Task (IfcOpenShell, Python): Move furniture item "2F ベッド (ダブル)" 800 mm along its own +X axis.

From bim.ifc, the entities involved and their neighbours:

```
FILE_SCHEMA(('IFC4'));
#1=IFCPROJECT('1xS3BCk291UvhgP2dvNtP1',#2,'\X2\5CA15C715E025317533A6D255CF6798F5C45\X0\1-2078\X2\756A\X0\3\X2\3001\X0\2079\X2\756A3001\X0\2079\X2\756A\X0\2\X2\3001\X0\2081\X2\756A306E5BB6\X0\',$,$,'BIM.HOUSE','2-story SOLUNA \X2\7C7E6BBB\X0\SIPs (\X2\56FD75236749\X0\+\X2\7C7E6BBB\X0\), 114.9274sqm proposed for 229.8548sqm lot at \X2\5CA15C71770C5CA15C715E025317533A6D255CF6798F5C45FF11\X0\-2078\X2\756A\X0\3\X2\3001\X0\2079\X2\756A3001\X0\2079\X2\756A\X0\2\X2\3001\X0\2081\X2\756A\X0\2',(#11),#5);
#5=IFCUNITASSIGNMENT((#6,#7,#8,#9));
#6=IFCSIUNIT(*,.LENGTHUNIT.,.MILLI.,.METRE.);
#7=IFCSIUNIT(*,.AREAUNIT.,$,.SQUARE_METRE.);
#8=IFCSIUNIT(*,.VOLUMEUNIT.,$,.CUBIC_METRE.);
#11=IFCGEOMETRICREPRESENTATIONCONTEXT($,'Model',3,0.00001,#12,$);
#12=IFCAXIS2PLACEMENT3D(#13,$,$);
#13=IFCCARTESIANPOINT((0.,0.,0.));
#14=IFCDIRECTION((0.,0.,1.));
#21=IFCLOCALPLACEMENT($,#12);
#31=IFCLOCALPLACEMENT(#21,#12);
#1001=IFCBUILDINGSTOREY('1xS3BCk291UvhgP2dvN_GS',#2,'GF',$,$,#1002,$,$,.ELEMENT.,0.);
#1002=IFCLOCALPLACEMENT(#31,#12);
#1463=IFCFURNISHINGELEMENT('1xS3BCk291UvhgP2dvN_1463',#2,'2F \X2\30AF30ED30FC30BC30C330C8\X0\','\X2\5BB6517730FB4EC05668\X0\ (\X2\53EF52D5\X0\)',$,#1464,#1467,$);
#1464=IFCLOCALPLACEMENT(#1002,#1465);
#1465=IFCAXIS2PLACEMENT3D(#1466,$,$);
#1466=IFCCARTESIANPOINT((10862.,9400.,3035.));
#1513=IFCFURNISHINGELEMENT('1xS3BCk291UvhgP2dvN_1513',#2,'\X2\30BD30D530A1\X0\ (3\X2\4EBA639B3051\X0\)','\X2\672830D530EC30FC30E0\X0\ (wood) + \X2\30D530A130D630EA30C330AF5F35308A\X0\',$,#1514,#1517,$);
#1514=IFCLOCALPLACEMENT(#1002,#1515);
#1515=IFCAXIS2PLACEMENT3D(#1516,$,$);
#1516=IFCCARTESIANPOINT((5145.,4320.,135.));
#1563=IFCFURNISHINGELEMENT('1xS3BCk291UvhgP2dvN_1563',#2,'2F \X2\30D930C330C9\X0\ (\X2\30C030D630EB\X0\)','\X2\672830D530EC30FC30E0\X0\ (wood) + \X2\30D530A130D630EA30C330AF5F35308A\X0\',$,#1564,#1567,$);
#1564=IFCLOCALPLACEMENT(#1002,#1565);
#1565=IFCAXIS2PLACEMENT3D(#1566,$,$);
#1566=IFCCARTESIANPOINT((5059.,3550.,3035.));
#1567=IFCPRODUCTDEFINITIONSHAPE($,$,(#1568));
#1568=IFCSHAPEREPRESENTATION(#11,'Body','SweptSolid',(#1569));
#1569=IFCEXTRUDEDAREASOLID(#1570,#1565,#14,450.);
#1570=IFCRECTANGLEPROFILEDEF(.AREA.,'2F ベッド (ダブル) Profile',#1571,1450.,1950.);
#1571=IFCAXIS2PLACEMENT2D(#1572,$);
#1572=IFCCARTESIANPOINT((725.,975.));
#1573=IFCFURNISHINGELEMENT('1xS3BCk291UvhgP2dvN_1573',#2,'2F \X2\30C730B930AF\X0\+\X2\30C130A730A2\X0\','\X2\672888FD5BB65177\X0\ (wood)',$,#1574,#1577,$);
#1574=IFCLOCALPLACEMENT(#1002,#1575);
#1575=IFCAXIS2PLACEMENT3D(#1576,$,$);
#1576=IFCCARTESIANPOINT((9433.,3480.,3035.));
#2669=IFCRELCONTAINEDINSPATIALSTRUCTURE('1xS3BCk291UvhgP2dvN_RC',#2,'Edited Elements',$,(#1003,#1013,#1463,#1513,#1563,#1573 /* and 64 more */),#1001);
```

```python
import ifcopenshell
import ifcopenshell.api.geometry
import ifcopenshell.util.placement
import ifcopenshell.util.unit

model = ifcopenshell.open("bim.ifc")
unit_scale = ifcopenshell.util.unit.calculate_unit_scale(model)

item = model.by_guid("1xS3BCk291UvhgP2dvN_1563")
matrix = ifcopenshell.util.placement.get_local_placement(item.ObjectPlacement)
matrix[:3, 3] += matrix[:3, 0] * 0.8 / unit_scale
ifcopenshell.api.geometry.edit_object_placement(model, product=item, matrix=matrix, is_si=False)

print(ifcopenshell.util.placement.get_local_placement(item.ObjectPlacement).round(3) + 0.0)

model.write("bim_rev.ifc")
```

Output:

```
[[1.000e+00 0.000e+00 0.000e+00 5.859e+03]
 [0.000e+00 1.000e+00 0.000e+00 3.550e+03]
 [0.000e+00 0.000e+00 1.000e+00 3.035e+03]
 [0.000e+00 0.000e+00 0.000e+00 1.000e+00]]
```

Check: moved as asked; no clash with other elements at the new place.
